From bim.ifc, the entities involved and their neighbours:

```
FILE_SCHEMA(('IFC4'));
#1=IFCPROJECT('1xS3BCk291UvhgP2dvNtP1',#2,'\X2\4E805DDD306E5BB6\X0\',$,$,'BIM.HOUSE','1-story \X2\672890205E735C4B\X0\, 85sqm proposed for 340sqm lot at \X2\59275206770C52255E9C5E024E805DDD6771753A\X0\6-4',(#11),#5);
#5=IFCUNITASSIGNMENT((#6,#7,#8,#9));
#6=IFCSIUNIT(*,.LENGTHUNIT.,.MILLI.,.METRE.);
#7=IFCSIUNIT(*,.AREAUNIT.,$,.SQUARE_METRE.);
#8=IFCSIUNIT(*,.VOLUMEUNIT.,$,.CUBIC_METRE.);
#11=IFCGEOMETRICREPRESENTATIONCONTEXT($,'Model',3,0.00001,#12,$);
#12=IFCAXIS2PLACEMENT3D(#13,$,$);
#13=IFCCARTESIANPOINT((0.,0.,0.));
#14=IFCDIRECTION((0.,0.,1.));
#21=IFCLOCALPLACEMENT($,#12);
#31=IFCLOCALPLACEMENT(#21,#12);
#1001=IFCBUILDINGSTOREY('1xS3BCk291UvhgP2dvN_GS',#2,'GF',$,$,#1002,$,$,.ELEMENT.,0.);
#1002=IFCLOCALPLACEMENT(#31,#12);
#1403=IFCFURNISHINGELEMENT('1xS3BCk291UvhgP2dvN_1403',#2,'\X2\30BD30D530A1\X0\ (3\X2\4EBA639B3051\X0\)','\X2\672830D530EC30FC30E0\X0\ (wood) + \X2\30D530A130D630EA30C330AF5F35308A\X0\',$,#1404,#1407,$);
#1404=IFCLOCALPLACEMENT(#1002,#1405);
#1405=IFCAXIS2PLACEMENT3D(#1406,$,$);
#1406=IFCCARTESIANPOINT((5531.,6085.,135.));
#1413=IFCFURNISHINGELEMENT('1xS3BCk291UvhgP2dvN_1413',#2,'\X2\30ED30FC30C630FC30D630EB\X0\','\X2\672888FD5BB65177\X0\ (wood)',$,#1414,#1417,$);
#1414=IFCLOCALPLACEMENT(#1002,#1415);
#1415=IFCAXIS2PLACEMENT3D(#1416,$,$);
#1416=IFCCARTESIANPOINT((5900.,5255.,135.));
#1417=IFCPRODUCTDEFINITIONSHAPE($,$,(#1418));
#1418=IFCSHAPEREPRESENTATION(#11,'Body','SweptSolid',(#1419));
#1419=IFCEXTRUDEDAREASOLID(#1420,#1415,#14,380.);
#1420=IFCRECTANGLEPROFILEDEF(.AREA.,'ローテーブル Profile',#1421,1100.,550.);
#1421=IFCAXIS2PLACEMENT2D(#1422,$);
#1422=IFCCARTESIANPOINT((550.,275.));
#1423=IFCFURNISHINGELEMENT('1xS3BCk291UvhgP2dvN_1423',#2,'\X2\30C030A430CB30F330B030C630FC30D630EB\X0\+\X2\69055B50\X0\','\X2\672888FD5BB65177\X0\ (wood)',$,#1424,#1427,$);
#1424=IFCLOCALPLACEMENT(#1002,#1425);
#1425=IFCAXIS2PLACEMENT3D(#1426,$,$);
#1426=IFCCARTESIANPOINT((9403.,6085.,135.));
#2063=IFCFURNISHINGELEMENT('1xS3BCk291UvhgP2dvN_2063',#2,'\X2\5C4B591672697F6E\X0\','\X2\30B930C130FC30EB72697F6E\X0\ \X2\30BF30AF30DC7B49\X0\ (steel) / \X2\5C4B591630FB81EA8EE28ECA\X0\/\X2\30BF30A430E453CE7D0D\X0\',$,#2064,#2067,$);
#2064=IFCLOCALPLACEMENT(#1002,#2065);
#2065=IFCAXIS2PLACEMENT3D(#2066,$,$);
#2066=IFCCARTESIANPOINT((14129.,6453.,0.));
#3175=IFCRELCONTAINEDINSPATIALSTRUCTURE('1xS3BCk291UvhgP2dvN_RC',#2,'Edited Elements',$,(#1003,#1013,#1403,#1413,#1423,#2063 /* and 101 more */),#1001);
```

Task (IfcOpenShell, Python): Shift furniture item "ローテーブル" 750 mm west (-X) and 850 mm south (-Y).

```python
import ifcopenshell
import ifcopenshell.api.geometry
import ifcopenshell.util.placement
import ifcopenshell.util.unit

model = ifcopenshell.open("bim.ifc")
unit_scale = ifcopenshell.util.unit.calculate_unit_scale(model)

item = model.by_guid("1xS3BCk291UvhgP2dvN_1413")
matrix = ifcopenshell.util.placement.get_local_placement(item.ObjectPlacement)
matrix[0, 3] -= 0.75 / unit_scale
matrix[1, 3] -= 0.85 / unit_scale
ifcopenshell.api.geometry.edit_object_placement(model, product=item, matrix=matrix, is_si=False)

print(ifcopenshell.util.placement.get_local_placement(item.ObjectPlacement).round(3) + 0.0)

model.write("bim_v2.ifc")
```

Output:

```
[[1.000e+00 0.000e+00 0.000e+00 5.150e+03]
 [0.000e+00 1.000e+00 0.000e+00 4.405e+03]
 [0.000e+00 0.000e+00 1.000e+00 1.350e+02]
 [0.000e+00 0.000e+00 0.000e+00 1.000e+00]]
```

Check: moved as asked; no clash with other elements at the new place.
